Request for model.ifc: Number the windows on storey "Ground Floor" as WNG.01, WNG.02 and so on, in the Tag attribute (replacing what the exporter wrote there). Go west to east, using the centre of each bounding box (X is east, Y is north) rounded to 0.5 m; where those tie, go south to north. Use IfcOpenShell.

First a look at what the model holds.

```python
import ifcopenshell
import ifcopenshell.util.element
import ifcopenshell.util.placement

model = ifcopenshell.open("model.ifc")
print(model.schema)
storey = next(s for s in model.by_type("IfcBuildingStorey") if s.Name == "Ground Floor")
windows = [e for e in ifcopenshell.util.element.get_decomposition(storey) if e.is_a("IfcWindow")]
for e in sorted(windows, key=lambda e: e.id()):
    origin = ifcopenshell.util.placement.get_local_placement(e.ObjectPlacement)[:3, 3]
    print(e.id(), e.Tag, e.Name, origin.round(2) + 0.0, sep=" | ")
```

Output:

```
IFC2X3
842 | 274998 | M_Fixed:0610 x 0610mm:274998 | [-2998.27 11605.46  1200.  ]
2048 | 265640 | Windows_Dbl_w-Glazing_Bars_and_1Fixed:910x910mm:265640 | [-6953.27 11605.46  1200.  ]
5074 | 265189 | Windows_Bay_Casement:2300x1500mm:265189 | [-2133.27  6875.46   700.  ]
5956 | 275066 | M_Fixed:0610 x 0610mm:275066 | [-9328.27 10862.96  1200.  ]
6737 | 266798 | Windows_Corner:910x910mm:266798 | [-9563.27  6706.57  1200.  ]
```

```python
import ifcopenshell
import ifcopenshell.geom
import ifcopenshell.util.element
import ifcopenshell.util.shape

model = ifcopenshell.open("model.ifc")
settings = ifcopenshell.geom.settings()
settings.set("use-world-coords", True)


def centre(element):
    shape = ifcopenshell.geom.create_shape(settings, element)
    return ifcopenshell.util.shape.get_bbox_centroid(shape.geometry)


storey = next(s for s in model.by_type("IfcBuildingStorey") if s.Name == "Ground Floor")
windows = [e for e in ifcopenshell.util.element.get_decomposition(storey) if e.is_a("IfcWindow")]

# Insertion points can sit at a corner or the storey origin, so sort by the geometry (in metres).
centres = {e: centre(e) for e in windows}
windows.sort(key=lambda e: (round(centres[e][0] / 0.5), centres[e][1]))

for i, e in enumerate(windows, start=1):
    number = f"WNG.{i:02d}"
    e.Tag = number
    print(e.id(), number)

model.write("model_updated.ifc")
```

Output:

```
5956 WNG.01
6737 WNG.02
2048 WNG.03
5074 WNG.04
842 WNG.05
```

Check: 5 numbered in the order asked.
